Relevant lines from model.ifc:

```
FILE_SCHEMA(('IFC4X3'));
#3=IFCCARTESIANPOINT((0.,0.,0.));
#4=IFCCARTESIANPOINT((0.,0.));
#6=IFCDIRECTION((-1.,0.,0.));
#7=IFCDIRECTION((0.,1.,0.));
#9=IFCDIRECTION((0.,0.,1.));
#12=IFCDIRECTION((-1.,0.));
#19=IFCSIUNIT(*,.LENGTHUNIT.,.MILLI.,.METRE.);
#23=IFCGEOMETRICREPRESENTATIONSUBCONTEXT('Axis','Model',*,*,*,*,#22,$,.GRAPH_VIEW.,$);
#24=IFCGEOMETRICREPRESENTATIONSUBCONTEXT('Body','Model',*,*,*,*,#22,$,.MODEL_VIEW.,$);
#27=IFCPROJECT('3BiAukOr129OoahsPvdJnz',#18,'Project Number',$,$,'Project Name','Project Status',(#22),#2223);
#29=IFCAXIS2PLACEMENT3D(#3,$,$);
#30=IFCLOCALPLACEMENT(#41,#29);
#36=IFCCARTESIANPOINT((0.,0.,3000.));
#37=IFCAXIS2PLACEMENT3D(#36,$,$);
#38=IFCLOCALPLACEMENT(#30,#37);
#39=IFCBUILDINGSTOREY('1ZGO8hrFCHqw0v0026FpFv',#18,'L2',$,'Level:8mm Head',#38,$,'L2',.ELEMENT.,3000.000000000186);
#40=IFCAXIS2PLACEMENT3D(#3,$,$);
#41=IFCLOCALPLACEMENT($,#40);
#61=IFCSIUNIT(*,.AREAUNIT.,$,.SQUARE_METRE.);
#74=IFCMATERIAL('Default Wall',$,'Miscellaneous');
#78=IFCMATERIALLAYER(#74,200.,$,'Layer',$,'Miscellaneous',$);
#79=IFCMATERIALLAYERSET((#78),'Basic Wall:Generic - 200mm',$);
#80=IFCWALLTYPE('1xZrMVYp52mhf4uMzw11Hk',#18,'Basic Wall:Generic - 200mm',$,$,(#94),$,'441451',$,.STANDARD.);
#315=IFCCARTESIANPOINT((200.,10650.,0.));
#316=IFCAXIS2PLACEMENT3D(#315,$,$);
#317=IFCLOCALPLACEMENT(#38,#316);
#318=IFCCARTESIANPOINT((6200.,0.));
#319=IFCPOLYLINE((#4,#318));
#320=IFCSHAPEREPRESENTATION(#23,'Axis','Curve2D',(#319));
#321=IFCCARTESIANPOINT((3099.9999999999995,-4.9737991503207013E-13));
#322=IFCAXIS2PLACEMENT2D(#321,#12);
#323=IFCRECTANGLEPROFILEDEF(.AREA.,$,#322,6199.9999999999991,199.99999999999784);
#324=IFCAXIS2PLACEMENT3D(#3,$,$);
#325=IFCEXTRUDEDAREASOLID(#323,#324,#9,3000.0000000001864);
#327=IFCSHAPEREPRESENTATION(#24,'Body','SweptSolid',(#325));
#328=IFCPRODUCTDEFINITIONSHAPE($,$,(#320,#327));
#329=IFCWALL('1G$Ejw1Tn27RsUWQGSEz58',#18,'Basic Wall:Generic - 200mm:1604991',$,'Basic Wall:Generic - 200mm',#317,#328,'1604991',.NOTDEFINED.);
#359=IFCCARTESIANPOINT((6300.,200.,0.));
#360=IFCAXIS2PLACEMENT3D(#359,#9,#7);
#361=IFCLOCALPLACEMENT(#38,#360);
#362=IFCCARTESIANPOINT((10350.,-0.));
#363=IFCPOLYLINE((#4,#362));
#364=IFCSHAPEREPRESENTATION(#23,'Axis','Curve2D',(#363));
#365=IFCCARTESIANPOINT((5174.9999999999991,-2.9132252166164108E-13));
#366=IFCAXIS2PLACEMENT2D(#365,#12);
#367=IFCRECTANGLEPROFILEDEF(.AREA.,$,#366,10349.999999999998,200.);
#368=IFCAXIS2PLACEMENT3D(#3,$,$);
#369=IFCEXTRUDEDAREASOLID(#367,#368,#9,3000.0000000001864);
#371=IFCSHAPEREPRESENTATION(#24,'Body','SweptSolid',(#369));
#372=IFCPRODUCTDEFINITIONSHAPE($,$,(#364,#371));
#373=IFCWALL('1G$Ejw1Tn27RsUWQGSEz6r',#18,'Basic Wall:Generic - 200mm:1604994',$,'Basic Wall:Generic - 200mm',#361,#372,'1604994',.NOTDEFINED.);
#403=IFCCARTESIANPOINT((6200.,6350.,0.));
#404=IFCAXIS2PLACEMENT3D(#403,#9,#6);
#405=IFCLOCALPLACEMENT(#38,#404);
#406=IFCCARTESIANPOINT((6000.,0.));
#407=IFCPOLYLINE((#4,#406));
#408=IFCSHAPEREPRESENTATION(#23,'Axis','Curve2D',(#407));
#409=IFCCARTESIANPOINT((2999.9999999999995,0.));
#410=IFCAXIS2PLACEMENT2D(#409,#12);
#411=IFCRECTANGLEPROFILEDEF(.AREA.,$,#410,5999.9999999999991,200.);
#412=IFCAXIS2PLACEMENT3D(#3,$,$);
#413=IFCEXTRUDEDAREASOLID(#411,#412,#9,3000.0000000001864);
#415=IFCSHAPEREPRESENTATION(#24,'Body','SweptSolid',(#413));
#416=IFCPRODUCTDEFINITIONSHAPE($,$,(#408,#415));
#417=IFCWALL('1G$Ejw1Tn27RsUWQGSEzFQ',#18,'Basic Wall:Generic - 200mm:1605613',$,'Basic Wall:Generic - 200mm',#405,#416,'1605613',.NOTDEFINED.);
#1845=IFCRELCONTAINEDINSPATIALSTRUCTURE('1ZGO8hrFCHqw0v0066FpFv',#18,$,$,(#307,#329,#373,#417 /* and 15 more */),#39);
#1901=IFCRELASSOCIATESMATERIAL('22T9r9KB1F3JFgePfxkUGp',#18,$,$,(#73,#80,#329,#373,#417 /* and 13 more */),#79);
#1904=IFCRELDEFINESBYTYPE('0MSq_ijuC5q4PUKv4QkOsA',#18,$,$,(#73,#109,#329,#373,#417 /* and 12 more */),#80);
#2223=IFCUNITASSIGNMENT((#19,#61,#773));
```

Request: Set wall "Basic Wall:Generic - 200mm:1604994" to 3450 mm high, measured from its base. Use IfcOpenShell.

```python
import ifcopenshell
import ifcopenshell.geom
import ifcopenshell.util.representation
import ifcopenshell.util.shape
import ifcopenshell.util.unit

model = ifcopenshell.open("model.ifc")
unit_scale = ifcopenshell.util.unit.calculate_unit_scale(model)
settings = ifcopenshell.geom.settings()


def volume(element):
    """Net volume in cubic metres, openings subtracted."""
    shape = ifcopenshell.geom.create_shape(settings, element)
    return ifcopenshell.util.shape.get_volume(shape.geometry)


wall = model.by_guid("1G$Ejw1Tn27RsUWQGSEz6r")
before = volume(wall)

body = ifcopenshell.util.representation.get_representation(wall, "Model", "Body")
solid = body.Items[0]
old_height = solid.Depth
solid.Depth = 3.45 / unit_scale
after = volume(wall)

print(f"height {old_height:g} -> {solid.Depth:g}, volume {before:.3f} -> {after:.3f} m3")

model.write("model_updated.ifc")
```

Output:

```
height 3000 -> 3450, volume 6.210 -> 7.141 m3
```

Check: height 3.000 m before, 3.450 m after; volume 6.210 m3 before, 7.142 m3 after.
